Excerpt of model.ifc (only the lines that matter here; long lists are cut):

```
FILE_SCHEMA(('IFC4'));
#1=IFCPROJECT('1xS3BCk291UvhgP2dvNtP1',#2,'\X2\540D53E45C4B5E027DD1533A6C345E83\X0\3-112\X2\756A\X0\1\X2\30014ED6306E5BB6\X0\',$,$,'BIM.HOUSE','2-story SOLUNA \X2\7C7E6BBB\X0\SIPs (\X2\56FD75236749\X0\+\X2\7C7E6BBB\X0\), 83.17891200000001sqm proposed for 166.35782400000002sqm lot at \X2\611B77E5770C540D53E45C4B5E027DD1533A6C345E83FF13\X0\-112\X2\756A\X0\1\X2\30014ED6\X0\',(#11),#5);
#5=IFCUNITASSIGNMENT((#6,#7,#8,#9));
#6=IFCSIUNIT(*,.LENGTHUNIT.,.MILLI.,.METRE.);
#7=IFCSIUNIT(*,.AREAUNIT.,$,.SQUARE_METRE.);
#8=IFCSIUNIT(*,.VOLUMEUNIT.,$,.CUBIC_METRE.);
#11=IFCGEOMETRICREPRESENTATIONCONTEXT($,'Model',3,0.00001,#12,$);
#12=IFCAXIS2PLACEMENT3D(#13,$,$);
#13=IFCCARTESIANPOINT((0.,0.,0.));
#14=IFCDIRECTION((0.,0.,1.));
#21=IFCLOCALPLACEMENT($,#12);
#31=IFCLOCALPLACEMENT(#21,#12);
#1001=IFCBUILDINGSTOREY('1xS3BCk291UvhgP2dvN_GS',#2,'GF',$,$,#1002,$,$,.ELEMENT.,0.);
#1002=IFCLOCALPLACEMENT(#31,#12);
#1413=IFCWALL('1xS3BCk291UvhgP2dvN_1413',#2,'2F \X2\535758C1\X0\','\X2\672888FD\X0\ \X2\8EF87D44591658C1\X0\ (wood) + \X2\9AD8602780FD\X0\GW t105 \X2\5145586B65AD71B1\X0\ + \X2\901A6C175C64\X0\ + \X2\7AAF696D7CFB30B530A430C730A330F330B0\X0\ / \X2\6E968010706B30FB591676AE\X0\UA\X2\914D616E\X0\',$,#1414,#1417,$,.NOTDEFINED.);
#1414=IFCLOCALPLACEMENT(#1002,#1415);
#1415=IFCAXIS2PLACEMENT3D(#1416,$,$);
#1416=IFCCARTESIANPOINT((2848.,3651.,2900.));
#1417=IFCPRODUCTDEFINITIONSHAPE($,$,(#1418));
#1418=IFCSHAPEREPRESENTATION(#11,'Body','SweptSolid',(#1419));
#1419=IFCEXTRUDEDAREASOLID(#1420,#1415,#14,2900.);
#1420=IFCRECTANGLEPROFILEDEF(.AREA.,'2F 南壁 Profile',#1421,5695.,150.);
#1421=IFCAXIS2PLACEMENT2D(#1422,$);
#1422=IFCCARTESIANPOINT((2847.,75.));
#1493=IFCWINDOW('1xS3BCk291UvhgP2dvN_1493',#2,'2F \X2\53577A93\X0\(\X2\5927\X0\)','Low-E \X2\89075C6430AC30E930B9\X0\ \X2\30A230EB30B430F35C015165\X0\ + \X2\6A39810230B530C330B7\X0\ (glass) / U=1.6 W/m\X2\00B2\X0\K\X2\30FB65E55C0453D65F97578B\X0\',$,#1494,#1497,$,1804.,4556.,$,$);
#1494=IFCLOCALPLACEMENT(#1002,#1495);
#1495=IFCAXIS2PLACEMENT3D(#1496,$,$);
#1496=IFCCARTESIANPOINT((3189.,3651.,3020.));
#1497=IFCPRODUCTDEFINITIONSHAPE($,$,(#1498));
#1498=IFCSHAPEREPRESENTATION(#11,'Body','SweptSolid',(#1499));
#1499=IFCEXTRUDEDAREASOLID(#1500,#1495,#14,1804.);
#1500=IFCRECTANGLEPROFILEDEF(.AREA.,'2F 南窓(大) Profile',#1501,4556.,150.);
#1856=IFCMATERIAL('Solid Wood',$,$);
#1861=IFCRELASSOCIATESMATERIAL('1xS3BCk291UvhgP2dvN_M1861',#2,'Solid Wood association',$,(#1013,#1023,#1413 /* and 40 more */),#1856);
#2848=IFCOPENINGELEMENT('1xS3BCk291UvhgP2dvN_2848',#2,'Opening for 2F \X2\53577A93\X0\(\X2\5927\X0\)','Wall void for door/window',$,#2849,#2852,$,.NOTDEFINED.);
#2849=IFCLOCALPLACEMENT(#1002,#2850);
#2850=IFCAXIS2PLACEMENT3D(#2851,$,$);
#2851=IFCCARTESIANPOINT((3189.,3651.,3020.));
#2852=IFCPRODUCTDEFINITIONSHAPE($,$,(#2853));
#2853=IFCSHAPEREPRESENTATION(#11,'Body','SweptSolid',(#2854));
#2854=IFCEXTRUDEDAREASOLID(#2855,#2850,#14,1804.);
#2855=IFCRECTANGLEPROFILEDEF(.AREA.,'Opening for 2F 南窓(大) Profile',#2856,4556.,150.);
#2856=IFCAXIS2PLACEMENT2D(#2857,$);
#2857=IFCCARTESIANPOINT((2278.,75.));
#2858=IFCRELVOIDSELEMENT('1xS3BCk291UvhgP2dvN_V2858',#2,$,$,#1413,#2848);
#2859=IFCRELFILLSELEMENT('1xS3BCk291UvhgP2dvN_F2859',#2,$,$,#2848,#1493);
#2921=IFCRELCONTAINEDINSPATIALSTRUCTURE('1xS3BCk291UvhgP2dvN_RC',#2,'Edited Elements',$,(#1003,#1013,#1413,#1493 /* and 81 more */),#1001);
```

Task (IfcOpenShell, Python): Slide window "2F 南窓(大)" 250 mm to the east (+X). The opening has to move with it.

```python
import ifcopenshell
import ifcopenshell.api.geometry
import ifcopenshell.util.placement

model = ifcopenshell.open("model.ifc")

window = model.by_id(1493)
opening = window.FillsVoids[0].RelatingOpeningElement
wall = opening.VoidsElements[0].RelatingBuildingElement

wall_matrix = ifcopenshell.util.placement.get_local_placement(wall.ObjectPlacement)
shift = wall_matrix[:3, 0] * 250.0
before = ifcopenshell.util.placement.get_local_placement(window.ObjectPlacement)[:3, 3].copy()

# The window is not placed relative to its opening, so move both.
for product in (opening, window):
    matrix = ifcopenshell.util.placement.get_local_placement(product.ObjectPlacement)
    matrix[:3, 3] += shift
    ifcopenshell.api.geometry.edit_object_placement(model, product=product, matrix=matrix, is_si=False)

after = ifcopenshell.util.placement.get_local_placement(window.ObjectPlacement)[:3, 3]
print("window moved by", (after - before).round(3) + 0.0)

model.write("model-out.ifc")
```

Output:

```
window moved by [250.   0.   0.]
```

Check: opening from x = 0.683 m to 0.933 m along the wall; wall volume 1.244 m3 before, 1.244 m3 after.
